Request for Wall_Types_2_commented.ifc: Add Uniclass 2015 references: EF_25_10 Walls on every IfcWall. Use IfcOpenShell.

First a look at what the model holds.

```python
import ifcopenshell

model = ifcopenshell.open("Wall_Types_2_commented.ifc")
print(model.schema)
print("classifications:", [c.Name for c in model.by_type("IfcClassification")])
for ifc_class in ("IfcDoor", "IfcRoof", "IfcStair", "IfcWall", "IfcWindow"):
    print(ifc_class, len(model.by_type(ifc_class)))
```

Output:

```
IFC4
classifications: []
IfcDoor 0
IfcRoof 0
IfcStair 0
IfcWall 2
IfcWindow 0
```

```python
import ifcopenshell
import ifcopenshell.api.classification

model = ifcopenshell.open("Wall_Types_2_commented.ifc")

system = ifcopenshell.api.classification.add_classification(model, classification="Uniclass 2015")

codes = {
    "IfcWall": ("EF_25_10", "Walls"),
}
for ifc_class, (code, name) in codes.items():
    products = model.by_type(ifc_class)
    ifcopenshell.api.classification.add_reference(
        model, products=products, classification=system, identification=code, name=name
    )
    print(code, len(products))

model.write("Wall_Types_2_commented_rev.ifc")
```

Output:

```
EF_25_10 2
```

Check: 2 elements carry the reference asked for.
